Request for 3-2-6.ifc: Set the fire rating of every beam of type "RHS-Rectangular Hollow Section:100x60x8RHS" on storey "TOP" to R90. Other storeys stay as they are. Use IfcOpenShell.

First a look at what the model holds.

```python
import ifcopenshell
import ifcopenshell.util.element

model = ifcopenshell.open("3-2-6.ifc")
print(model.schema)
storey = next(s for s in model.by_type("IfcBuildingStorey") if s.Name == "TOP")
beams = [e for e in ifcopenshell.util.element.get_decomposition(storey) if e.is_a("IfcBeam")]
seen = {}
for e in beams:
    element_type = ifcopenshell.util.element.get_type(e)
    key = (element_type.Name if element_type != e and element_type else None, ifcopenshell.util.element.get_pset(e, "Pset_BeamCommon", "FireRating"))
    seen[key] = seen.get(key, 0) + 1
for (name, value), count in sorted(seen.items(), key=str):
    print(count, "x", name, "|", value)
```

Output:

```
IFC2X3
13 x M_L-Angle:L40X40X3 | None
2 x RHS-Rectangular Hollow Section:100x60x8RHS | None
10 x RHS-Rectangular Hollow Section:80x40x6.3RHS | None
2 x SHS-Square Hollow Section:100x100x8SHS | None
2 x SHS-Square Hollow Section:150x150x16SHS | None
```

```python
import ifcopenshell
import ifcopenshell.api.pset
import ifcopenshell.util.element

model = ifcopenshell.open("3-2-6.ifc")

storey = next(s for s in model.by_type("IfcBuildingStorey") if s.Name == "TOP")
beams = [e for e in ifcopenshell.util.element.get_decomposition(storey) if e.is_a("IfcBeam")]

count = 0
for e in beams:
    element_type = ifcopenshell.util.element.get_type(e)
    if element_type in (None, e) or element_type.Name != "RHS-Rectangular Hollow Section:100x60x8RHS":
        continue
    # add_pset returns the element's existing set when there is one.
    pset = ifcopenshell.api.pset.add_pset(model, product=e, name="Pset_BeamCommon")
    ifcopenshell.api.pset.edit_pset(model, pset=pset, properties={"FireRating": "R90"})
    count += 1

print(count, "beams updated")

model.write("3-2-6_edited.ifc")
```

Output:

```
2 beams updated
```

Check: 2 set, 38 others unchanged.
